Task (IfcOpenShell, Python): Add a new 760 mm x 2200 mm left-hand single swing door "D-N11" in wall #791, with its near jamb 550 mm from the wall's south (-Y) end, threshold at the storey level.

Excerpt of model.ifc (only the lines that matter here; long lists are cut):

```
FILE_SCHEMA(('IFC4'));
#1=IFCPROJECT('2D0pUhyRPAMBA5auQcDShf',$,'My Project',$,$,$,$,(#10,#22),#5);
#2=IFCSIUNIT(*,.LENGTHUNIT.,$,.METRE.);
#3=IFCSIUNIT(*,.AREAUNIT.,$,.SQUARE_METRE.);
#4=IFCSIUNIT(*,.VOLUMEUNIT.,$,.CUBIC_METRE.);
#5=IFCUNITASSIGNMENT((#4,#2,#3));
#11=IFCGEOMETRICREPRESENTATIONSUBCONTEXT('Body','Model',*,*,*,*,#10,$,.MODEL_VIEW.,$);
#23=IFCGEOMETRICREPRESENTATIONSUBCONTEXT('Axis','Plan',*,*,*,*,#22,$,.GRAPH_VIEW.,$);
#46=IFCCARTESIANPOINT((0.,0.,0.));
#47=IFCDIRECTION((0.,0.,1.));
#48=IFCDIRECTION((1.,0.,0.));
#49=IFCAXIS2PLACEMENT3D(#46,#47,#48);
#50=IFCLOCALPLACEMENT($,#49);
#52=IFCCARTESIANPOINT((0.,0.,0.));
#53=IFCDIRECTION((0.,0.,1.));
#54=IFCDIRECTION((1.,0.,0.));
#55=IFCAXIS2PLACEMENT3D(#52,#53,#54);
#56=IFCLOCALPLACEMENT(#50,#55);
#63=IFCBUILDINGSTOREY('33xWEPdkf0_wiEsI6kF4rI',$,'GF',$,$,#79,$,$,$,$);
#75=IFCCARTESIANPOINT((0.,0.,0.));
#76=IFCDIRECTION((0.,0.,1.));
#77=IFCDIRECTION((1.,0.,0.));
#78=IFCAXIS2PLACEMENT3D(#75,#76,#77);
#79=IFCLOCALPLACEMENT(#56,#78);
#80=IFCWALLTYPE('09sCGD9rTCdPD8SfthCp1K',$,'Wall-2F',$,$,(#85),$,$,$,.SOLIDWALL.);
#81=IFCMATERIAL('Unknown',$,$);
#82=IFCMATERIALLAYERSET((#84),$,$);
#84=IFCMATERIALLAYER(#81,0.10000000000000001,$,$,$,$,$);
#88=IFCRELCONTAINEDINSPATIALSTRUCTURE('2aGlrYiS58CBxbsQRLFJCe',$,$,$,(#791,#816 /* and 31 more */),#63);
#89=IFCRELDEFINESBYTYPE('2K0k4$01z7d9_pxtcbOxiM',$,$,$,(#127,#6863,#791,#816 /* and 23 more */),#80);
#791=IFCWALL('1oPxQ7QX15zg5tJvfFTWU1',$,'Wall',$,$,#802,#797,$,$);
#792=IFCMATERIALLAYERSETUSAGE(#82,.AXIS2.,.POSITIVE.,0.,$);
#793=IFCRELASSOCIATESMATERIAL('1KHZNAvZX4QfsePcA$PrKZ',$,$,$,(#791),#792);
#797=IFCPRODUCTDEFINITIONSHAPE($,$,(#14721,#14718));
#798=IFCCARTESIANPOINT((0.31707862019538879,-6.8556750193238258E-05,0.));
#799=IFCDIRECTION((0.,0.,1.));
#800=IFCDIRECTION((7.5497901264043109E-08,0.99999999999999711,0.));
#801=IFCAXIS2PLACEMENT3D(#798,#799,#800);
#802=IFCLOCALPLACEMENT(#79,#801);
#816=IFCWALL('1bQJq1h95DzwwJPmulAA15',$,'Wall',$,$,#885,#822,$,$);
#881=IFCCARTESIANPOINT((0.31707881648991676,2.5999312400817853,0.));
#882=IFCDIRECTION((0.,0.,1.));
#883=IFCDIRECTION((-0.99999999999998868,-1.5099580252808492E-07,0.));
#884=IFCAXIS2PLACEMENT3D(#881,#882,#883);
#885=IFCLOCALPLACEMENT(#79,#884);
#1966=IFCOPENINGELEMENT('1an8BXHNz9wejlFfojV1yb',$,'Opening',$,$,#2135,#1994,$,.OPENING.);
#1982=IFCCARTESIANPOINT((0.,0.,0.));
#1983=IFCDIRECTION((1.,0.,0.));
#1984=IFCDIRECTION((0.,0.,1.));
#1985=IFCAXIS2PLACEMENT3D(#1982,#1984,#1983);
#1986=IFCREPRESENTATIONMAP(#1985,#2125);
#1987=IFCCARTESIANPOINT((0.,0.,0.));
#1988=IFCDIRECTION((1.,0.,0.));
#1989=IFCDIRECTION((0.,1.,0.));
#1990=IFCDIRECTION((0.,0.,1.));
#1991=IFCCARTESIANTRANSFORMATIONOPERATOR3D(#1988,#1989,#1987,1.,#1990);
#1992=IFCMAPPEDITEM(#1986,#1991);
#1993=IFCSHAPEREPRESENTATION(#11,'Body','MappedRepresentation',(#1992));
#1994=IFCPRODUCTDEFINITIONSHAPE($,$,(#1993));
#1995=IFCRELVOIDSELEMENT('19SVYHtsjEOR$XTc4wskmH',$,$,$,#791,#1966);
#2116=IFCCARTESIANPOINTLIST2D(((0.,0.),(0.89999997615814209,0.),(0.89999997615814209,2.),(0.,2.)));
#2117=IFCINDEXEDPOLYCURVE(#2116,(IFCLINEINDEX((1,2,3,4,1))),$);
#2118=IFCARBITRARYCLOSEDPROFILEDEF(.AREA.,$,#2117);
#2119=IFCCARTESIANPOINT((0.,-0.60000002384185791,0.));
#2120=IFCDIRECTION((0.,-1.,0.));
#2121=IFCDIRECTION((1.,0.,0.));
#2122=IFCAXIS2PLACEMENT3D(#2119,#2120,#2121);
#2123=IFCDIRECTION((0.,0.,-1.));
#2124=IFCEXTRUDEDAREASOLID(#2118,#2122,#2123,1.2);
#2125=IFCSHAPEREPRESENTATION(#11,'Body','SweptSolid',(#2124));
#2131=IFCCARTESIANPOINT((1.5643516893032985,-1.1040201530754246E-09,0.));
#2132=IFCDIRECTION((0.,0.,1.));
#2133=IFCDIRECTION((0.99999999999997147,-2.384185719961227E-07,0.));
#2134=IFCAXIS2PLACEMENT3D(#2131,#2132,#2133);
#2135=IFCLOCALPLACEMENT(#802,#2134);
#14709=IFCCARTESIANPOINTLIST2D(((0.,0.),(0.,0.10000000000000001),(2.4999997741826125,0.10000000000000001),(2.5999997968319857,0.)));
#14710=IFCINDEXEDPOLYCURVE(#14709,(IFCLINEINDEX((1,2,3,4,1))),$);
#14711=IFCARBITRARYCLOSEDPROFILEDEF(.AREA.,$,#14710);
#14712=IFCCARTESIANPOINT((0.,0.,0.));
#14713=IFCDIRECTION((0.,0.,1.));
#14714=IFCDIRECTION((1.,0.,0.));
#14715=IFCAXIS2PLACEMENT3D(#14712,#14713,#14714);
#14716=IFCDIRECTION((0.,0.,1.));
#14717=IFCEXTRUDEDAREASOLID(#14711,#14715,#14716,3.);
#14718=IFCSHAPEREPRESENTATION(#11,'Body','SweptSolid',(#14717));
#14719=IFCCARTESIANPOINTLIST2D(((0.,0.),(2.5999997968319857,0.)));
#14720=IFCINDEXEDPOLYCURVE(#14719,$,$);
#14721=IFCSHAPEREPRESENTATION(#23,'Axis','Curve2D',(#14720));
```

```python
import numpy as np
import ifcopenshell
import ifcopenshell.api.feature
import ifcopenshell.api.geometry
import ifcopenshell.api.root
import ifcopenshell.api.spatial
import ifcopenshell.geom
import ifcopenshell.util.element
import ifcopenshell.util.placement
import ifcopenshell.util.representation
import ifcopenshell.util.shape
import ifcopenshell.util.unit

model = ifcopenshell.open("model.ifc")
unit_scale = ifcopenshell.util.unit.calculate_unit_scale(model)
settings = ifcopenshell.geom.settings()


def volume(element):
    """Net volume in cubic metres, openings subtracted."""
    shape = ifcopenshell.geom.create_shape(settings, element)
    return ifcopenshell.util.shape.get_volume(shape.geometry)


wall = model.by_guid("1oPxQ7QX15zg5tJvfFTWU1")
storey = ifcopenshell.util.element.get_container(wall, ifc_class="IfcBuildingStorey")
context = ifcopenshell.util.representation.get_context(model, "Model", "Body", "MODEL_VIEW")
before = volume(wall)

width, height, from_end, sill = 0.76, 2.2, 0.55, 0.0  # metres

# The wall runs along its own X axis, and the end named is its -X end.
wall_shape = ifcopenshell.geom.create_shape(settings, wall)
x, y, z = ifcopenshell.util.shape.get_vertices(wall_shape.geometry).T
start = x.min() + from_end
face, thickness = float(y.min()), float(y.max() - y.min())
wall_matrix = ifcopenshell.util.placement.get_local_placement(wall.ObjectPlacement)
level = ifcopenshell.util.placement.get_local_placement(storey.ObjectPlacement)[2, 3]


def in_wall(x, y):
    """Placement at x, y metres in the wall's axes, at sill height."""
    matrix = wall_matrix.copy()
    matrix[:, 3] = wall_matrix @ np.array([x / unit_scale, y / unit_scale, 0.0, 1.0])
    matrix[2, 3] = level + sill / unit_scale
    return matrix


# Opening: a box that overshoots both wall faces by 50 mm.
opening = ifcopenshell.api.root.create_entity(model, ifc_class="IfcOpeningElement", predefined_type="OPENING")
box = ifcopenshell.api.geometry.add_wall_representation(
    model, context=context, length=width, height=height, thickness=thickness + 0.1
)
ifcopenshell.api.geometry.assign_representation(model, product=opening, representation=box)
ifcopenshell.api.geometry.edit_object_placement(model, product=opening, matrix=in_wall(start, face - 0.05), is_si=False)
ifcopenshell.api.feature.add_feature(model, feature=opening, element=wall)

door = ifcopenshell.api.root.create_entity(model, ifc_class="IfcDoor", name="D-N11", predefined_type="DOOR")
door.OverallWidth, door.OverallHeight = width / unit_scale, height / unit_scale
door.OperationType = "SINGLE_SWING_LEFT"
body = ifcopenshell.api.geometry.add_door_representation(
    model,
    context=context,
    overall_width=door.OverallWidth,
    overall_height=door.OverallHeight,
    operation_type="SINGLE_SWING_LEFT",
    lining_properties={"LiningDepth": thickness / unit_scale, "ThresholdDepth": thickness / unit_scale},
)
ifcopenshell.api.geometry.assign_representation(model, product=door, representation=body)
ifcopenshell.api.spatial.assign_container(model, products=[door], relating_structure=storey)
ifcopenshell.api.feature.add_filling(model, opening=opening, element=door)

# The lining spans the wall, so the door starts at the wall face.
ifcopenshell.api.geometry.edit_object_placement(model, product=door, matrix=in_wall(start, face), is_si=False)

after = volume(wall)

print(f"wall volume {before:.3f} -> {after:.3f} m3")

model.write("model-out.ifc")
```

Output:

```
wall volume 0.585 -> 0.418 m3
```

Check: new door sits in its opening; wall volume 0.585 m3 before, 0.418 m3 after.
